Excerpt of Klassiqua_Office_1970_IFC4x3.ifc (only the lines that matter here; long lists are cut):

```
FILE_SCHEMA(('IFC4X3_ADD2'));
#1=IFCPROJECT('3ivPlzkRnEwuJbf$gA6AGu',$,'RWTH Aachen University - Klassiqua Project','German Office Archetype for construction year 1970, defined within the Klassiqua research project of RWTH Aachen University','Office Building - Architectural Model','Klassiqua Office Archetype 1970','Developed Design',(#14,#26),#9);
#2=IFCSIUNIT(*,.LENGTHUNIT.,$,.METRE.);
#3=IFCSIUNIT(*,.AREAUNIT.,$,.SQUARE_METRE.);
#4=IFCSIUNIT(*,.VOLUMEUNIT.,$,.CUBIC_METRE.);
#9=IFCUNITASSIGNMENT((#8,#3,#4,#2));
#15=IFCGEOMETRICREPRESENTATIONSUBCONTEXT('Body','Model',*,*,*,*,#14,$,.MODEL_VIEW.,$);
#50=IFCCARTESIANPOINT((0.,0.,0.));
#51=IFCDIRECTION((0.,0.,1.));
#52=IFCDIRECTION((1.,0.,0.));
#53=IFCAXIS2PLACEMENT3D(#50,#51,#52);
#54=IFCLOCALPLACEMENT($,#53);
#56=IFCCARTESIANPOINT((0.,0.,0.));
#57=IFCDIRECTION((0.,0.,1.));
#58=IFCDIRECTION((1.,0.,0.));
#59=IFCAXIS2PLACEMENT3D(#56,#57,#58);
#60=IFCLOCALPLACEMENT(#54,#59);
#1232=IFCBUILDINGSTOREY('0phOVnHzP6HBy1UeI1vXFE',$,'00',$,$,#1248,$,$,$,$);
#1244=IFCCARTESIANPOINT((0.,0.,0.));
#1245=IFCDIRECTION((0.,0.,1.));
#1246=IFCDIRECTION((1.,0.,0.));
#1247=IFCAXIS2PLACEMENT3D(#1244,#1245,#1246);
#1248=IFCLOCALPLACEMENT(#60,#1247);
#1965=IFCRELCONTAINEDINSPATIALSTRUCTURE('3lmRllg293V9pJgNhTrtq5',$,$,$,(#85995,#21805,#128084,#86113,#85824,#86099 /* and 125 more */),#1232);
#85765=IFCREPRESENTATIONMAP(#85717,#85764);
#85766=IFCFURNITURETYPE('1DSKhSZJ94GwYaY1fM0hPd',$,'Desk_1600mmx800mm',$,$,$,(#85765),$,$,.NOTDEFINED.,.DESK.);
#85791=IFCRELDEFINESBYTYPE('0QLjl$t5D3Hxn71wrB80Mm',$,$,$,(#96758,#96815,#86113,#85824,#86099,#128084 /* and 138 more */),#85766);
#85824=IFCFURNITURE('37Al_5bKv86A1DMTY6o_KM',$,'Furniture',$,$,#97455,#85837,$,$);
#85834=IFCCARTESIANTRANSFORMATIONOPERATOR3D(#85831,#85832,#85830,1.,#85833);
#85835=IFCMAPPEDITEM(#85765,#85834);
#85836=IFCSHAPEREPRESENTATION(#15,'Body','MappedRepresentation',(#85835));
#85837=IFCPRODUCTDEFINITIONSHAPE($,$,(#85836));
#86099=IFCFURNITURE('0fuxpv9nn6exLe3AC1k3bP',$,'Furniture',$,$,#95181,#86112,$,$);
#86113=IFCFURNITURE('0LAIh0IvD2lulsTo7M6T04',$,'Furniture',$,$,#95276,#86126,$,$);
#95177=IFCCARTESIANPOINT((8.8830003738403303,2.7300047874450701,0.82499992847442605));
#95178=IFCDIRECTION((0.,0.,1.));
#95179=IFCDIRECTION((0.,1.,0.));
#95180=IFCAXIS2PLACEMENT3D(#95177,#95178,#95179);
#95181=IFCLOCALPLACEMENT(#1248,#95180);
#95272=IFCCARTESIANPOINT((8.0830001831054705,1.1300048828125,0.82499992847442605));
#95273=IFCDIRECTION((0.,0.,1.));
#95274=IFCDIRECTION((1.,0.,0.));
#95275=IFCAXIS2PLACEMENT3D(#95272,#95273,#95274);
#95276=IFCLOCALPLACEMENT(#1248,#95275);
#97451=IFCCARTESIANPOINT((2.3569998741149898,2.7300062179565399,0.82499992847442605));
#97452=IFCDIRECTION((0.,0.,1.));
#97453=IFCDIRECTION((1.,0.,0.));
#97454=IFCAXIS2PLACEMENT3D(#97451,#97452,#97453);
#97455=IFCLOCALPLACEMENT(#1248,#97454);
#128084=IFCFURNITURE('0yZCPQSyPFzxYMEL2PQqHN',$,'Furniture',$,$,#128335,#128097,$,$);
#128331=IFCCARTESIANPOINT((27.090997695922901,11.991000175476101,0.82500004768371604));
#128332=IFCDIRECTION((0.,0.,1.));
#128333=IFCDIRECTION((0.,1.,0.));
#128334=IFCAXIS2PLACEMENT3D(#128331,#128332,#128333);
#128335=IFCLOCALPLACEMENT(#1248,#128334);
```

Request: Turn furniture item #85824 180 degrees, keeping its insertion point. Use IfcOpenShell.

```python
import ifcopenshell
import ifcopenshell.api.geometry
import ifcopenshell.util.placement

model = ifcopenshell.open("Klassiqua_Office_1970_IFC4x3.ifc")

item = model.by_id(85824)
matrix = ifcopenshell.util.placement.get_local_placement(item.ObjectPlacement)
matrix = matrix @ ifcopenshell.util.placement.rotation(180, "Z")
ifcopenshell.api.geometry.edit_object_placement(model, product=item, matrix=matrix, is_si=False)

print(ifcopenshell.util.placement.get_local_placement(item.ObjectPlacement).round(3) + 0.0)

model.write("Klassiqua_Office_1970_IFC4x3_updated.ifc")
```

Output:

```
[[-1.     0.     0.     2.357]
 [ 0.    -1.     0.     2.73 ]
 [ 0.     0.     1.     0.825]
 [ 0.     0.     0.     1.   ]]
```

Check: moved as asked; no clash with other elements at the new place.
